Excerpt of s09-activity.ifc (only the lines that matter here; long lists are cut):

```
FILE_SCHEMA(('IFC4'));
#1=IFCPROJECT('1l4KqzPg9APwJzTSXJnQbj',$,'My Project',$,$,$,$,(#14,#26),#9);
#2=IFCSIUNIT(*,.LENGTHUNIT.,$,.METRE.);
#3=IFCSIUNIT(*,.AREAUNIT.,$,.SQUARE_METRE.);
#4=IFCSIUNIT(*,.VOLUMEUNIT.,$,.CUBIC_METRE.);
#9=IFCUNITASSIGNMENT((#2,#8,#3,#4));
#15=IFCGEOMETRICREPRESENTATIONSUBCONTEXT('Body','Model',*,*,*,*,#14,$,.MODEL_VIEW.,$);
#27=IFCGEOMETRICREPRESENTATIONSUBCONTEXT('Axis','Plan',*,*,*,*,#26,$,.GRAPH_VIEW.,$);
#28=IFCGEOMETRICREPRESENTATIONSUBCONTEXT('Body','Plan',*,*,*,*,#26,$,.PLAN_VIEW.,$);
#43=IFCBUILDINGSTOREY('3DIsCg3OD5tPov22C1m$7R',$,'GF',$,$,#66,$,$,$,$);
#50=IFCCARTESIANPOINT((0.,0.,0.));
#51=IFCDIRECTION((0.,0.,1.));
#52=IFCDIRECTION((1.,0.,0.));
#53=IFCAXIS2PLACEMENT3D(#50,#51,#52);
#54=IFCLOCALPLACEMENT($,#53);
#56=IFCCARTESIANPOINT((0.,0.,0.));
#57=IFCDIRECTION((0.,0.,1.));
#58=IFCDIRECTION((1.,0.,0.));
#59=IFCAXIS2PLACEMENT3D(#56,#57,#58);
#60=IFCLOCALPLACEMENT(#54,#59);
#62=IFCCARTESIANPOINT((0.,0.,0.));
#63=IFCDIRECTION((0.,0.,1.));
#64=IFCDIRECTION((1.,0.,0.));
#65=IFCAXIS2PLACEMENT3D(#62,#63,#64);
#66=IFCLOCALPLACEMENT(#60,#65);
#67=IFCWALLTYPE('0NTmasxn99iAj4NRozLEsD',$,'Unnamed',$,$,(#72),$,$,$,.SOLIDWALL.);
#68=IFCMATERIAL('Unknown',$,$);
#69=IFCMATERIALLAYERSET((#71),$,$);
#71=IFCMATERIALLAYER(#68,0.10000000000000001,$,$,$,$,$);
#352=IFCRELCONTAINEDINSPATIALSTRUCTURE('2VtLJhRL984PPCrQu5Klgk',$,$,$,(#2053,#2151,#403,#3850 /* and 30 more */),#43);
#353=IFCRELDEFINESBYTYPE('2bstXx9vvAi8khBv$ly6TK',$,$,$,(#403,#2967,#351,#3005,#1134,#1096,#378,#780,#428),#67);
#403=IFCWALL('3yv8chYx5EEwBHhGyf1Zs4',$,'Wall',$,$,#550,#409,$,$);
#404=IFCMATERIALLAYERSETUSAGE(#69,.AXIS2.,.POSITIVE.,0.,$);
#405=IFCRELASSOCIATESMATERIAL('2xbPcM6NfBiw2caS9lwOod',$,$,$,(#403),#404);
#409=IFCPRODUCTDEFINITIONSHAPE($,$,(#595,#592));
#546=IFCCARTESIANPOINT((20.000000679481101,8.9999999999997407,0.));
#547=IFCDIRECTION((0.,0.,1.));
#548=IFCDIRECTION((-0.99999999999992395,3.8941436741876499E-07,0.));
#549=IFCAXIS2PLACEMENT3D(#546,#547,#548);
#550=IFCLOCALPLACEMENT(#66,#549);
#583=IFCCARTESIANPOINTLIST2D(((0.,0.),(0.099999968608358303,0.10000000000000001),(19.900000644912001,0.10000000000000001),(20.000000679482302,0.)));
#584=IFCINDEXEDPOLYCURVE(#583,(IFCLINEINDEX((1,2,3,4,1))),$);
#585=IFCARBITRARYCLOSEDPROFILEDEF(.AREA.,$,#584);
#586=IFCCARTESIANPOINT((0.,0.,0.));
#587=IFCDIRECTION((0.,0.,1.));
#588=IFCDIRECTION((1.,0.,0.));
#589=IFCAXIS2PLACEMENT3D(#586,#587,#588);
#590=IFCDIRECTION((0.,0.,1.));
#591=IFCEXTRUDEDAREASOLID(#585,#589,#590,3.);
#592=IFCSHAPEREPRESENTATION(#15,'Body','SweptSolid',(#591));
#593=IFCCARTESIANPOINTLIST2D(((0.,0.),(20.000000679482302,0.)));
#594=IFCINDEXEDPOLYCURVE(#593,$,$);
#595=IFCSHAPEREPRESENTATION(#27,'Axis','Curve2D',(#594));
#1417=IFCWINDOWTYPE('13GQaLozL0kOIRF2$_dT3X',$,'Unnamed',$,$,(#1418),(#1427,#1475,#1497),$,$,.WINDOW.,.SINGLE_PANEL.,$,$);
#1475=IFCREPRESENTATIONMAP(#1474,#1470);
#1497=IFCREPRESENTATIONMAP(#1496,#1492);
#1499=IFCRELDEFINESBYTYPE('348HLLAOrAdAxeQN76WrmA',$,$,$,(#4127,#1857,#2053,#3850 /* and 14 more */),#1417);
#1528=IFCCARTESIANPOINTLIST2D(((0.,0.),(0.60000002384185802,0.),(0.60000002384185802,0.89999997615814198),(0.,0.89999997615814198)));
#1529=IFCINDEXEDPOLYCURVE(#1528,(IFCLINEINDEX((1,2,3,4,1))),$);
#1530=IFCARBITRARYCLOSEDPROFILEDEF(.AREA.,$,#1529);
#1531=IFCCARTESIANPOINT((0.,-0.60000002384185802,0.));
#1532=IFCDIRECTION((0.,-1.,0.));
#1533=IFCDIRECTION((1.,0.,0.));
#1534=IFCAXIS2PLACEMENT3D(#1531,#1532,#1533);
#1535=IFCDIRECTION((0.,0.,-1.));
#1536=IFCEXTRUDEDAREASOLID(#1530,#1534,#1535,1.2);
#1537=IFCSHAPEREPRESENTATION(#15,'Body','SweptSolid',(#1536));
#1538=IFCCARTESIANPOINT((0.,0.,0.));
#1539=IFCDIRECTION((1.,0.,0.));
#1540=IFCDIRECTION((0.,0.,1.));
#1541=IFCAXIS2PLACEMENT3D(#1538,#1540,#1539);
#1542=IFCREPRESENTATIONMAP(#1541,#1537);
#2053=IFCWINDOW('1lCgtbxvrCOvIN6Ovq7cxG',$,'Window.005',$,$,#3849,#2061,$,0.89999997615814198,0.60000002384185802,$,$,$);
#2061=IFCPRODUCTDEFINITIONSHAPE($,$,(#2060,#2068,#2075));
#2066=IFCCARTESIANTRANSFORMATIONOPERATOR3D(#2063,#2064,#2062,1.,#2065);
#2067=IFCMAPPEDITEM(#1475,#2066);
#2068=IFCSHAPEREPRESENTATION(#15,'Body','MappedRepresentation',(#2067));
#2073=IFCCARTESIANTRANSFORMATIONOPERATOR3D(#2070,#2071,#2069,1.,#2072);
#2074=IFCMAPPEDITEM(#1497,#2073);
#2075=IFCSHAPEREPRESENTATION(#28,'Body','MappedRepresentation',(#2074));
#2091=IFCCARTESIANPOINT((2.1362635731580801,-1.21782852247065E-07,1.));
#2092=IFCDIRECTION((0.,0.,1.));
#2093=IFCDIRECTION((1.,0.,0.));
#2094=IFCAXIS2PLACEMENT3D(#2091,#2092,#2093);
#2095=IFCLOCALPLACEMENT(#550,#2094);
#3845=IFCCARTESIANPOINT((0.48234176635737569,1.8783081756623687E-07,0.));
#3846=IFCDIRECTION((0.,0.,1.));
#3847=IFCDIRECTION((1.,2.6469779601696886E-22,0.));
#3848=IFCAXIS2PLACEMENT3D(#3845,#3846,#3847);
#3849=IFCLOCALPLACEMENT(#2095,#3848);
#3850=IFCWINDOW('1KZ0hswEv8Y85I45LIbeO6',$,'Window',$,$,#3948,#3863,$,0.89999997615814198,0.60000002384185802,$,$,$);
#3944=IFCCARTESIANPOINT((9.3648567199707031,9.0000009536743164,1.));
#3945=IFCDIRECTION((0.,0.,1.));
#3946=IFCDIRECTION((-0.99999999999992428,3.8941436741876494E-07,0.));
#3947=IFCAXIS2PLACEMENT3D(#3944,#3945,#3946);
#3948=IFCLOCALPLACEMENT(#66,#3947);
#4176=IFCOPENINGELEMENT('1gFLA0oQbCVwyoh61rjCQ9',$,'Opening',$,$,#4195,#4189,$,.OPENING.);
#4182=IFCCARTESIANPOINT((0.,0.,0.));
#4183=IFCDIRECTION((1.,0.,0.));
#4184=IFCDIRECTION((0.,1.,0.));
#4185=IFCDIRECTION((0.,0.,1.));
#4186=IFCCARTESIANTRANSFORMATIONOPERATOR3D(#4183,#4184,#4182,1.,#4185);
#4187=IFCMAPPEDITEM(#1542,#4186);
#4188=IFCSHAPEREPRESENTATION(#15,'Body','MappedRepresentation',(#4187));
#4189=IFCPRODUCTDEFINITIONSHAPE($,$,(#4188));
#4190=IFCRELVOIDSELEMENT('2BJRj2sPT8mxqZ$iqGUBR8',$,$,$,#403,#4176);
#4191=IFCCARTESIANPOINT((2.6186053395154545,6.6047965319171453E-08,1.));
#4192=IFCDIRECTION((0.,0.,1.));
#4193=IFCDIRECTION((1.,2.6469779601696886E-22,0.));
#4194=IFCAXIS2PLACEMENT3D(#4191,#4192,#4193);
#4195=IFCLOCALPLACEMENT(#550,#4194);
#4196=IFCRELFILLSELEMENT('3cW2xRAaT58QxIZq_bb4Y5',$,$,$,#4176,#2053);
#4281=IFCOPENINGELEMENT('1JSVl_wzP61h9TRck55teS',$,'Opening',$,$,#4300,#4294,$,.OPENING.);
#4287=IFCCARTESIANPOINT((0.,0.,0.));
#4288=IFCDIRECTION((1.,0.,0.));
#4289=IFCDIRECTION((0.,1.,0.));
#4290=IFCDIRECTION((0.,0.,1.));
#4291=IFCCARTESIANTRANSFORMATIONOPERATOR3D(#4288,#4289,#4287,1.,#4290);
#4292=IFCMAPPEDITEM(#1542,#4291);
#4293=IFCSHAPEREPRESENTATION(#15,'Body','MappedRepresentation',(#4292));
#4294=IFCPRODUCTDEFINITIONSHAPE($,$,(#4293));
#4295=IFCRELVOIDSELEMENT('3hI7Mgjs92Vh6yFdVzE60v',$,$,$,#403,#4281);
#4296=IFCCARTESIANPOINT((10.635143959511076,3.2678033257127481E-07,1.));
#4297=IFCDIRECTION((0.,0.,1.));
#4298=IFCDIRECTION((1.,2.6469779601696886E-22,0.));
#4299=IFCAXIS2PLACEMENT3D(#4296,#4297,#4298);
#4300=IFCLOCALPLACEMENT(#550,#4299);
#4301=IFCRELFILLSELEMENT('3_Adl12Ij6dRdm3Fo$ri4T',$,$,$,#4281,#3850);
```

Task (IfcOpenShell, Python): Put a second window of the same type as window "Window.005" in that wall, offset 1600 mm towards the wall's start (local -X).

```python
import ifcopenshell
import ifcopenshell.api.feature
import ifcopenshell.api.geometry
import ifcopenshell.api.root
import ifcopenshell.geom
import ifcopenshell.util.element
import ifcopenshell.util.placement
import ifcopenshell.util.shape
import ifcopenshell.util.unit

model = ifcopenshell.open("s09-activity.ifc")
unit_scale = ifcopenshell.util.unit.calculate_unit_scale(model)
settings = ifcopenshell.geom.settings()


def volume(element):
    """Net volume in cubic metres, openings subtracted."""
    shape = ifcopenshell.geom.create_shape(settings, element)
    return ifcopenshell.util.shape.get_volume(shape.geometry)


window = model.by_id(2053)
opening = window.FillsVoids[0].RelatingOpeningElement
wall = opening.VoidsElements[0].RelatingBuildingElement
before = volume(wall)
shift = ifcopenshell.util.placement.get_local_placement(wall.ObjectPlacement)[:3, 0] * -1.6 / unit_scale

# copy_class copies the void relationship, type, container and properties, but no geometry.
new_opening = ifcopenshell.api.root.copy_class(model, product=opening)
new_opening.Representation = ifcopenshell.util.element.copy_deep(
    model, opening.Representation, exclude=["IfcGeometricRepresentationContext", "IfcRepresentationMap"]
)
new_window = ifcopenshell.api.root.copy_class(model, product=window)
new_window.Representation = ifcopenshell.util.element.copy_deep(
    model, window.Representation, exclude=["IfcGeometricRepresentationContext", "IfcRepresentationMap"]
)
ifcopenshell.api.feature.add_filling(model, opening=new_opening, element=new_window)

for old, new in ((opening, new_opening), (window, new_window)):
    matrix = ifcopenshell.util.placement.get_local_placement(old.ObjectPlacement)
    matrix[:3, 3] += shift
    ifcopenshell.api.geometry.edit_object_placement(model, product=new, matrix=matrix, is_si=False)

after = volume(wall)

print(f"wall volume {before:.3f} -> {after:.3f} m3")

model.write("s09-activity_rev.ifc")
```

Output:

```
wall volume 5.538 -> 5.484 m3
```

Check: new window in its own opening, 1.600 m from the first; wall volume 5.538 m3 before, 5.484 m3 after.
